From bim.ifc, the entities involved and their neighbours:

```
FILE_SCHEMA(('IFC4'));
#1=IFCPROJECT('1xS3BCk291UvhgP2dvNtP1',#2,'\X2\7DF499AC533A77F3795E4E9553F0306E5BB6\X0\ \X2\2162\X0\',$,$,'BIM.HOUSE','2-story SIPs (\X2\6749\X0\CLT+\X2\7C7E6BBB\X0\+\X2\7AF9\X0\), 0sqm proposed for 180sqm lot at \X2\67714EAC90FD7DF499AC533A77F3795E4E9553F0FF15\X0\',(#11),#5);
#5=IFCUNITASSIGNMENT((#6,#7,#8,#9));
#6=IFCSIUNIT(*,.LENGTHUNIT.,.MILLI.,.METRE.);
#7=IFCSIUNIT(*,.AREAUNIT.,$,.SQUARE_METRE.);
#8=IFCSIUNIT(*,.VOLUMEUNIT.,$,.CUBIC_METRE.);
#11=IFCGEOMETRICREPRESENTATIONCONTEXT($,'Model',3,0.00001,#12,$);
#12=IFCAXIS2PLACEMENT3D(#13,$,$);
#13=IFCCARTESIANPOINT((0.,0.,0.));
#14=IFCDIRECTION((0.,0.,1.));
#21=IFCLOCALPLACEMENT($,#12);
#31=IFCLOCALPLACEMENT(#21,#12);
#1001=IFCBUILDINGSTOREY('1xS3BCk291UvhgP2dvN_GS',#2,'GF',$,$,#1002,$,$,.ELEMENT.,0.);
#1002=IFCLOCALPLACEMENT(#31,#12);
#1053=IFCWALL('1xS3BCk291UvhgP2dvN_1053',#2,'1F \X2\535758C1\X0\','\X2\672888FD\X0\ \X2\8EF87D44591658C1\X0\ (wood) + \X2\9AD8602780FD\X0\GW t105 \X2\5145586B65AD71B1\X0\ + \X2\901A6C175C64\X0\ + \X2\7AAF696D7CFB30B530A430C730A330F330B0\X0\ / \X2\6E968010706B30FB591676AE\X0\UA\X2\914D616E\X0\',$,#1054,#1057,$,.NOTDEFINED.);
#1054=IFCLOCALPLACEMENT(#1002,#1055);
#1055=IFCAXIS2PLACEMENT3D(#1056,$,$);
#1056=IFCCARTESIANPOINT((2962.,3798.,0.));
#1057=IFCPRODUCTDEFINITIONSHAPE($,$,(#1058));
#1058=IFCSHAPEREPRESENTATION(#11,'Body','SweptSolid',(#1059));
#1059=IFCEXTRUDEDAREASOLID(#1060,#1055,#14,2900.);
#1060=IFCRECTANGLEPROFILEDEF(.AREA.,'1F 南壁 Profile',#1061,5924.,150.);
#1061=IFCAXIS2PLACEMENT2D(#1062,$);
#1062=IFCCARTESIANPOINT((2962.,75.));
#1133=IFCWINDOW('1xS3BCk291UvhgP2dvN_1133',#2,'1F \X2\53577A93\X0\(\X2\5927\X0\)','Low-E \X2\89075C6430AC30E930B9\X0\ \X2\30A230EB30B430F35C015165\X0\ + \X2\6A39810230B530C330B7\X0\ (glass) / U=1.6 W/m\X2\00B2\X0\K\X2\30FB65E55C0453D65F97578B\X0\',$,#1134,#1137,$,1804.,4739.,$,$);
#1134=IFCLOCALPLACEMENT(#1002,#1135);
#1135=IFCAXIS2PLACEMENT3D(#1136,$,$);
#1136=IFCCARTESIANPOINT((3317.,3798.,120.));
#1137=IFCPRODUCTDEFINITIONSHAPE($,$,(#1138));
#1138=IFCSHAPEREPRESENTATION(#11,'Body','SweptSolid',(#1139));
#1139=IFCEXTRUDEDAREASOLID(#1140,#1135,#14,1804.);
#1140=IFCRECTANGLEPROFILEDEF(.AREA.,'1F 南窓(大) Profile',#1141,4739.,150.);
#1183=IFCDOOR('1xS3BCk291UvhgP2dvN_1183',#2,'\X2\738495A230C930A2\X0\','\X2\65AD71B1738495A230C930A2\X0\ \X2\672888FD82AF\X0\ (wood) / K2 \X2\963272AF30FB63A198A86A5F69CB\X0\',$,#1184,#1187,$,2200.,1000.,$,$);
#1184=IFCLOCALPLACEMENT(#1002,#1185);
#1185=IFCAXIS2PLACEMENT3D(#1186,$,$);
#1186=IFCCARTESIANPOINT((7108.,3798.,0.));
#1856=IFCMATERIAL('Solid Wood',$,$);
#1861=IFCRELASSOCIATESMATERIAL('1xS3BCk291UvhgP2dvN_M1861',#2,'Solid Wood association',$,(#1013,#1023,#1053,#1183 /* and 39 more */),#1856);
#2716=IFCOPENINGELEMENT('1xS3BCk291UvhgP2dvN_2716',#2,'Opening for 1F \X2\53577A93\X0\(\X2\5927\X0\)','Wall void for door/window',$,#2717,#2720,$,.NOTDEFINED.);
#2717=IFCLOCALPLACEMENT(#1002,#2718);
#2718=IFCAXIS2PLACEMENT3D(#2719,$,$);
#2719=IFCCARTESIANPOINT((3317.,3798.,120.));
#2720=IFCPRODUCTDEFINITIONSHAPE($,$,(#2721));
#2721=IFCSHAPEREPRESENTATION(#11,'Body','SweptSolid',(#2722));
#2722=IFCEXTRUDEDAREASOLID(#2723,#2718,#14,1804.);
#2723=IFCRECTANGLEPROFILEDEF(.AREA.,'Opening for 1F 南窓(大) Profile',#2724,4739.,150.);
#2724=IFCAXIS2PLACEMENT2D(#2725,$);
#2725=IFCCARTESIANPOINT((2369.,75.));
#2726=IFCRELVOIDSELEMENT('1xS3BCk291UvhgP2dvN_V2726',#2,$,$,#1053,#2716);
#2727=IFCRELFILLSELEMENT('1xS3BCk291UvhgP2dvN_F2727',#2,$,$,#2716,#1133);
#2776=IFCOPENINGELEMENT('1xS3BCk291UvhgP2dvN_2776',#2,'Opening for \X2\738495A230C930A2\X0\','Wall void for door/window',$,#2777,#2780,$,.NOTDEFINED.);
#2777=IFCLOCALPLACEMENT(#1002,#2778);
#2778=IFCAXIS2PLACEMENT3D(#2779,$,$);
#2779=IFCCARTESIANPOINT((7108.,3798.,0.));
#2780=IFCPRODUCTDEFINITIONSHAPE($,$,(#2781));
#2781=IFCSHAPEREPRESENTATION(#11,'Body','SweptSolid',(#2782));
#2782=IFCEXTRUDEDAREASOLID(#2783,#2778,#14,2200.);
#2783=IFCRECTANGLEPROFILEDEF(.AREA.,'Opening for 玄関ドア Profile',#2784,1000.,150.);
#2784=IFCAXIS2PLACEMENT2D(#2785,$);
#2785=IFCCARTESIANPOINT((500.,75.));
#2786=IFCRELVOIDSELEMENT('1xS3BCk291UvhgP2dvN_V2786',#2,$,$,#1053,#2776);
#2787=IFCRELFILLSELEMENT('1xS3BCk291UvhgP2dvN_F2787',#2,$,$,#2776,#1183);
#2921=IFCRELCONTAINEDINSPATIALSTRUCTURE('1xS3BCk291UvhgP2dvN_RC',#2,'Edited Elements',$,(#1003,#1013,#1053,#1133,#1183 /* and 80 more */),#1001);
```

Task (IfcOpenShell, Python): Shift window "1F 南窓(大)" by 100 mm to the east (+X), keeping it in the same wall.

```python
import ifcopenshell
import ifcopenshell.api.geometry
import ifcopenshell.util.placement

model = ifcopenshell.open("bim.ifc")

window = model.by_id(1133)
opening = window.FillsVoids[0].RelatingOpeningElement
wall = opening.VoidsElements[0].RelatingBuildingElement

wall_matrix = ifcopenshell.util.placement.get_local_placement(wall.ObjectPlacement)
shift = wall_matrix[:3, 0] * 100.0
before = ifcopenshell.util.placement.get_local_placement(window.ObjectPlacement)[:3, 3].copy()

# The window is not placed relative to its opening, so move both.
for product in (opening, window):
    matrix = ifcopenshell.util.placement.get_local_placement(product.ObjectPlacement)
    matrix[:3, 3] += shift
    ifcopenshell.api.geometry.edit_object_placement(model, product=product, matrix=matrix, is_si=False)

after = ifcopenshell.util.placement.get_local_placement(window.ObjectPlacement)[:3, 3]
print("window moved by", (after - before).round(3) + 0.0)

model.write("bim-out.ifc")
```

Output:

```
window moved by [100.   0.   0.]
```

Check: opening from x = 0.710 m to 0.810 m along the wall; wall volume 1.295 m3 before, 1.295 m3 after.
